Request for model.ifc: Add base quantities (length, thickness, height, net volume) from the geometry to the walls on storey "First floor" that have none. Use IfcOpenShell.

First a look at what the model holds.

```python
import ifcopenshell
import ifcopenshell.util.element
import ifcopenshell.util.unit

model = ifcopenshell.open("model.ifc")
print(model.schema)
for unit_type in ("LENGTHUNIT", "AREAUNIT", "VOLUMEUNIT"):
    print(unit_type, ifcopenshell.util.unit.calculate_unit_scale(model, unit_type))
storey = next(s for s in model.by_type("IfcBuildingStorey") if s.Name == "First floor")
walls = [e for e in ifcopenshell.util.element.get_decomposition(storey) if e.is_a("IfcWall")]
for e in sorted(walls, key=lambda e: e.id()):
    print(e.id(), e.is_a(), e.Name, list(ifcopenshell.util.element.get_psets(e, qtos_only=True)), sep=" | ")
```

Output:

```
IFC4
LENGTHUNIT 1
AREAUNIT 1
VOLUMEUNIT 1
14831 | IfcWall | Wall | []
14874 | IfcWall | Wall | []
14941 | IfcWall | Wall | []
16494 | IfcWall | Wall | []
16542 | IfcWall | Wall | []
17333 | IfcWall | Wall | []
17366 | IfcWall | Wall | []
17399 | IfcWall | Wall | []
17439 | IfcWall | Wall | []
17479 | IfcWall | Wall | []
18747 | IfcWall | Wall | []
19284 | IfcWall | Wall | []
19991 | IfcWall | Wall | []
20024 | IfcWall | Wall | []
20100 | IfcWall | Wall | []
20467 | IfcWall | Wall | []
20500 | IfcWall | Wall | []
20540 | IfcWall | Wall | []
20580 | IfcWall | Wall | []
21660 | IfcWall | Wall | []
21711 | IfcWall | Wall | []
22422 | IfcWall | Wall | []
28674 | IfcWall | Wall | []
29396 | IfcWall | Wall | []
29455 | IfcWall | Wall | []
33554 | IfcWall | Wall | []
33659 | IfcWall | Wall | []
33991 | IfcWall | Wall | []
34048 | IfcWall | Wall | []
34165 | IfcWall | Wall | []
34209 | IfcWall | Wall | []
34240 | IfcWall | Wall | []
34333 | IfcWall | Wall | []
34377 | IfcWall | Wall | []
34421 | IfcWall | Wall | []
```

```python
import ifcopenshell
import ifcopenshell.api.pset
import ifcopenshell.geom
import ifcopenshell.util.element
import ifcopenshell.util.shape
import ifcopenshell.util.unit

model = ifcopenshell.open("model.ifc")
unit_scale = ifcopenshell.util.unit.calculate_unit_scale(model)
volume_scale = ifcopenshell.util.unit.calculate_unit_scale(model, "VOLUMEUNIT")
settings = ifcopenshell.geom.settings()

storey = next(s for s in model.by_type("IfcBuildingStorey") if s.Name == "First floor")
walls = [e for e in ifcopenshell.util.element.get_decomposition(storey) if e.is_a("IfcWall")]

for e in sorted(walls, key=lambda e: e.id()):
    if ifcopenshell.util.element.get_psets(e, qtos_only=True, should_inherit=False):
        continue
    # Geometry comes back in metres, in the element's own axes.
    shape = ifcopenshell.geom.create_shape(settings, e)
    values = {
        "Length": ifcopenshell.util.shape.get_x(shape.geometry) / unit_scale,
        "Width": ifcopenshell.util.shape.get_y(shape.geometry) / unit_scale,
        "Height": ifcopenshell.util.shape.get_z(shape.geometry) / unit_scale,
        "NetVolume": ifcopenshell.util.shape.get_volume(shape.geometry) / volume_scale,
    }
    qto = ifcopenshell.api.pset.add_qto(model, product=e, name="Qto_WallBaseQuantities")
    ifcopenshell.api.pset.edit_qto(model, qto=qto, properties=values)
    print(e.id(), {k: round(v, 3) for k, v in values.items()})

model.write("model_edited.ifc")
```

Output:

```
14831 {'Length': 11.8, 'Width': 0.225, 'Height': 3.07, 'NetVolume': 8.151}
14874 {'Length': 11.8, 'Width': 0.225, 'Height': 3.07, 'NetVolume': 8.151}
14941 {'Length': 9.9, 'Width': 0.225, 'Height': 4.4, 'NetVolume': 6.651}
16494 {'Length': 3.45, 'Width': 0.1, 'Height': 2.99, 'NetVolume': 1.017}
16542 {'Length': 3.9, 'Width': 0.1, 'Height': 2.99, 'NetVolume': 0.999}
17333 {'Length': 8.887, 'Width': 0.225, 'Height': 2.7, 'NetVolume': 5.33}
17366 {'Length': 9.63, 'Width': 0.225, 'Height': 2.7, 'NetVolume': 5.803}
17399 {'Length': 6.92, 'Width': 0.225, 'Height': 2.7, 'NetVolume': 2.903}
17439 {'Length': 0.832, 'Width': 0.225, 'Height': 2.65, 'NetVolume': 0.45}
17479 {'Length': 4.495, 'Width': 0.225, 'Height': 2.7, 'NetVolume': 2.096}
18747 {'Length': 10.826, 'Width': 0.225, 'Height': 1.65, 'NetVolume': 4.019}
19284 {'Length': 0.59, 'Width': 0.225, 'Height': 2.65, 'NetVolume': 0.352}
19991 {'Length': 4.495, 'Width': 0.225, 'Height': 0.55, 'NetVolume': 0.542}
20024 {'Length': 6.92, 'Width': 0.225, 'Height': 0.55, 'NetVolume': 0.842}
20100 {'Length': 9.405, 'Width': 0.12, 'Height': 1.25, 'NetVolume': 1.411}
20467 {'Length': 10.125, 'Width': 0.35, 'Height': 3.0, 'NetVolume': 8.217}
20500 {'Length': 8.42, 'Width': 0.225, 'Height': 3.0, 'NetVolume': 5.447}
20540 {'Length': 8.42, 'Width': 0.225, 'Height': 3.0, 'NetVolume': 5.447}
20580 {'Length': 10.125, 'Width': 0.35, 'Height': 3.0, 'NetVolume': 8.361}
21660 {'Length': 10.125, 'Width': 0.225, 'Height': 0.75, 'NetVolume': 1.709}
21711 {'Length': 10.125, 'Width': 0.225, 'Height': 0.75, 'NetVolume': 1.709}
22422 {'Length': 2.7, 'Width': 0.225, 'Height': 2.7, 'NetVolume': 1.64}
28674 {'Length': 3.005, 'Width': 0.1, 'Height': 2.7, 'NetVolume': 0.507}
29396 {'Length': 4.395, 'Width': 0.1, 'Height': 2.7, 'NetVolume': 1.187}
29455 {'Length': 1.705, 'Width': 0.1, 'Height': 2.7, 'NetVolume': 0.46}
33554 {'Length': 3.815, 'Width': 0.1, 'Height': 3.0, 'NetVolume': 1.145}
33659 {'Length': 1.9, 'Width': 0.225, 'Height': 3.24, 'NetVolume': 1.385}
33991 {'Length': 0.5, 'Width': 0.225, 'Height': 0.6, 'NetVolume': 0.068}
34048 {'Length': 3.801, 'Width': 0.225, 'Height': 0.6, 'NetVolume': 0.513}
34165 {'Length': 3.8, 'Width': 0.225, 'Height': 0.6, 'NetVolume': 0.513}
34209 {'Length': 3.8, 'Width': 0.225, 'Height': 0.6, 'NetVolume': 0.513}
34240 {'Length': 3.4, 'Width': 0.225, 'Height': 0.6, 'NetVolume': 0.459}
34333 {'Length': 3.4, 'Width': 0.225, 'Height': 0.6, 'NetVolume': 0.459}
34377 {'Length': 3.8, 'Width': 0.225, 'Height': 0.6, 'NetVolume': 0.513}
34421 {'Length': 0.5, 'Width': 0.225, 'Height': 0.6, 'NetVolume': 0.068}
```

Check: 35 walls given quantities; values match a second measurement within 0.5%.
